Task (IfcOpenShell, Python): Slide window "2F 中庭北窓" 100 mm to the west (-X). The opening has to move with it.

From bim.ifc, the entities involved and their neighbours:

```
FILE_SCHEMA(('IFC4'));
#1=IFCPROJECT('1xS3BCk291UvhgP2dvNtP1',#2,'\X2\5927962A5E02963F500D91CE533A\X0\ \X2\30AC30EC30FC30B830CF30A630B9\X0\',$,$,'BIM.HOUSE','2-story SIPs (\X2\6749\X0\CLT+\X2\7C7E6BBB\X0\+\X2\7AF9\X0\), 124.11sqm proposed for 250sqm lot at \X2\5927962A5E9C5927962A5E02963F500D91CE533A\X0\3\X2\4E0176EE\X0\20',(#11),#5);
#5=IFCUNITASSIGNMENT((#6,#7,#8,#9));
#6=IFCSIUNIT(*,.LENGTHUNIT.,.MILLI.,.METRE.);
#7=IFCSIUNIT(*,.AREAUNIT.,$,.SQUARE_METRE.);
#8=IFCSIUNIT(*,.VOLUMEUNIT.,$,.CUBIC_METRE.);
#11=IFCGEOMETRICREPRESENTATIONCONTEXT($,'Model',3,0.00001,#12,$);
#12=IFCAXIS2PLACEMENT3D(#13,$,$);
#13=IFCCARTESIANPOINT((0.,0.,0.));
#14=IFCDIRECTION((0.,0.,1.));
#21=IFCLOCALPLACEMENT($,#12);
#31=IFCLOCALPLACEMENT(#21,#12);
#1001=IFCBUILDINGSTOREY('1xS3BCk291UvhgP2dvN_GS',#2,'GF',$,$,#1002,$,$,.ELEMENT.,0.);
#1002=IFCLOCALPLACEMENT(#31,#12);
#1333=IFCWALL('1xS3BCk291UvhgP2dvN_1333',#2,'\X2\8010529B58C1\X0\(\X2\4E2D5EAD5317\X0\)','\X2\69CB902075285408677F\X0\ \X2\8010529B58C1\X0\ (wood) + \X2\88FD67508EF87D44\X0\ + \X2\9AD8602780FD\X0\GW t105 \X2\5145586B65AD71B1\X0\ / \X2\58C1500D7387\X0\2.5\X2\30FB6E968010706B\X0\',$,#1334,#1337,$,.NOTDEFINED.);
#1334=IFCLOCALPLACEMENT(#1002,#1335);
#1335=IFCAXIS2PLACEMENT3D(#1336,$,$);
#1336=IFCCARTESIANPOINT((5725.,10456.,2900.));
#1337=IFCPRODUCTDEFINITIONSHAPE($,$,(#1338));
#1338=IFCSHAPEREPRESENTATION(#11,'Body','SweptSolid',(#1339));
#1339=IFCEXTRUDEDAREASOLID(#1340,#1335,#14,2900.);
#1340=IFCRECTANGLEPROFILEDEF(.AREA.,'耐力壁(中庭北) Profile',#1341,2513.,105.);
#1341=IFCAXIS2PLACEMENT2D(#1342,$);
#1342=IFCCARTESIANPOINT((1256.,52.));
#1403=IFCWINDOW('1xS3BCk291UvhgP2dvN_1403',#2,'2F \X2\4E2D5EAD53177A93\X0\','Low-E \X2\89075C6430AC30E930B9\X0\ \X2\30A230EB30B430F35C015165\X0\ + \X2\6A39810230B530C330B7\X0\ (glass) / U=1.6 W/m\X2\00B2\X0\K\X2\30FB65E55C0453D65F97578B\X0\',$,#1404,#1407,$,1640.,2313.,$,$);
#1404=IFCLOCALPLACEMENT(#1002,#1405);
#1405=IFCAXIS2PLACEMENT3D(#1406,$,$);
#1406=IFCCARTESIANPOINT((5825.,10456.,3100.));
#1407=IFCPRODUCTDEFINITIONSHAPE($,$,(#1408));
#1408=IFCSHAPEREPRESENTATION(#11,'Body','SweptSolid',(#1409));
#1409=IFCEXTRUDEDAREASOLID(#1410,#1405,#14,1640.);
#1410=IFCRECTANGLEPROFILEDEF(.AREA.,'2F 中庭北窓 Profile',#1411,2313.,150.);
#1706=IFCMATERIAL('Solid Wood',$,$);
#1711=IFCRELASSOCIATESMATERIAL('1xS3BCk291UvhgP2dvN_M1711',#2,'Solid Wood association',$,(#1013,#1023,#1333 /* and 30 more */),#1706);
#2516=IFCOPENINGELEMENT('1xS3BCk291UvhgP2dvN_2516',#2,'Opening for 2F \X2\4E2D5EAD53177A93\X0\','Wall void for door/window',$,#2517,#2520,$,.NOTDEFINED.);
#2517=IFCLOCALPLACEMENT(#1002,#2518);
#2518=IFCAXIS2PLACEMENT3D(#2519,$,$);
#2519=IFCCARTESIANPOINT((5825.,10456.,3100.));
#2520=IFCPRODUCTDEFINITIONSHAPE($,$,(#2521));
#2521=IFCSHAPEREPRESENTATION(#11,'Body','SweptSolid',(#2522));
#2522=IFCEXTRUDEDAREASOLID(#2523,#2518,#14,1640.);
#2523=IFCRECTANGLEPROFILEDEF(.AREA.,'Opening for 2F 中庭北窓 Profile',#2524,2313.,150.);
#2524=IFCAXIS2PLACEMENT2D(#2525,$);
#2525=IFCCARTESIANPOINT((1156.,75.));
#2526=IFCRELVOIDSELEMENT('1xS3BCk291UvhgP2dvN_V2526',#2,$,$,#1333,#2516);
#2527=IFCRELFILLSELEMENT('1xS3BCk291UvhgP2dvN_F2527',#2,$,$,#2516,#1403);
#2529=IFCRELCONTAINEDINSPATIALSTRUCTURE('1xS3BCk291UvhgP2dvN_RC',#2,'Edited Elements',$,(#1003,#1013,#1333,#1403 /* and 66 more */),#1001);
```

```python
import ifcopenshell
import ifcopenshell.api.geometry
import ifcopenshell.util.placement

model = ifcopenshell.open("bim.ifc")

window = model.by_guid("1xS3BCk291UvhgP2dvN_1403")
opening = window.FillsVoids[0].RelatingOpeningElement
wall = opening.VoidsElements[0].RelatingBuildingElement

wall_matrix = ifcopenshell.util.placement.get_local_placement(wall.ObjectPlacement)
shift = wall_matrix[:3, 0] * -100.0
before = ifcopenshell.util.placement.get_local_placement(window.ObjectPlacement)[:3, 3].copy()

# The window is not placed relative to its opening, so move both.
for product in (opening, window):
    matrix = ifcopenshell.util.placement.get_local_placement(product.ObjectPlacement)
    matrix[:3, 3] += shift
    ifcopenshell.api.geometry.edit_object_placement(model, product=product, matrix=matrix, is_si=False)

after = ifcopenshell.util.placement.get_local_placement(window.ObjectPlacement)[:3, 3]
print("window moved by", (after - before).round(3) + 0.0)

model.write("bim_updated.ifc")
```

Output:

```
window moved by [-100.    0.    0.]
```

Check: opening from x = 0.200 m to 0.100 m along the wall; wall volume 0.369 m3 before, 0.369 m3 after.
